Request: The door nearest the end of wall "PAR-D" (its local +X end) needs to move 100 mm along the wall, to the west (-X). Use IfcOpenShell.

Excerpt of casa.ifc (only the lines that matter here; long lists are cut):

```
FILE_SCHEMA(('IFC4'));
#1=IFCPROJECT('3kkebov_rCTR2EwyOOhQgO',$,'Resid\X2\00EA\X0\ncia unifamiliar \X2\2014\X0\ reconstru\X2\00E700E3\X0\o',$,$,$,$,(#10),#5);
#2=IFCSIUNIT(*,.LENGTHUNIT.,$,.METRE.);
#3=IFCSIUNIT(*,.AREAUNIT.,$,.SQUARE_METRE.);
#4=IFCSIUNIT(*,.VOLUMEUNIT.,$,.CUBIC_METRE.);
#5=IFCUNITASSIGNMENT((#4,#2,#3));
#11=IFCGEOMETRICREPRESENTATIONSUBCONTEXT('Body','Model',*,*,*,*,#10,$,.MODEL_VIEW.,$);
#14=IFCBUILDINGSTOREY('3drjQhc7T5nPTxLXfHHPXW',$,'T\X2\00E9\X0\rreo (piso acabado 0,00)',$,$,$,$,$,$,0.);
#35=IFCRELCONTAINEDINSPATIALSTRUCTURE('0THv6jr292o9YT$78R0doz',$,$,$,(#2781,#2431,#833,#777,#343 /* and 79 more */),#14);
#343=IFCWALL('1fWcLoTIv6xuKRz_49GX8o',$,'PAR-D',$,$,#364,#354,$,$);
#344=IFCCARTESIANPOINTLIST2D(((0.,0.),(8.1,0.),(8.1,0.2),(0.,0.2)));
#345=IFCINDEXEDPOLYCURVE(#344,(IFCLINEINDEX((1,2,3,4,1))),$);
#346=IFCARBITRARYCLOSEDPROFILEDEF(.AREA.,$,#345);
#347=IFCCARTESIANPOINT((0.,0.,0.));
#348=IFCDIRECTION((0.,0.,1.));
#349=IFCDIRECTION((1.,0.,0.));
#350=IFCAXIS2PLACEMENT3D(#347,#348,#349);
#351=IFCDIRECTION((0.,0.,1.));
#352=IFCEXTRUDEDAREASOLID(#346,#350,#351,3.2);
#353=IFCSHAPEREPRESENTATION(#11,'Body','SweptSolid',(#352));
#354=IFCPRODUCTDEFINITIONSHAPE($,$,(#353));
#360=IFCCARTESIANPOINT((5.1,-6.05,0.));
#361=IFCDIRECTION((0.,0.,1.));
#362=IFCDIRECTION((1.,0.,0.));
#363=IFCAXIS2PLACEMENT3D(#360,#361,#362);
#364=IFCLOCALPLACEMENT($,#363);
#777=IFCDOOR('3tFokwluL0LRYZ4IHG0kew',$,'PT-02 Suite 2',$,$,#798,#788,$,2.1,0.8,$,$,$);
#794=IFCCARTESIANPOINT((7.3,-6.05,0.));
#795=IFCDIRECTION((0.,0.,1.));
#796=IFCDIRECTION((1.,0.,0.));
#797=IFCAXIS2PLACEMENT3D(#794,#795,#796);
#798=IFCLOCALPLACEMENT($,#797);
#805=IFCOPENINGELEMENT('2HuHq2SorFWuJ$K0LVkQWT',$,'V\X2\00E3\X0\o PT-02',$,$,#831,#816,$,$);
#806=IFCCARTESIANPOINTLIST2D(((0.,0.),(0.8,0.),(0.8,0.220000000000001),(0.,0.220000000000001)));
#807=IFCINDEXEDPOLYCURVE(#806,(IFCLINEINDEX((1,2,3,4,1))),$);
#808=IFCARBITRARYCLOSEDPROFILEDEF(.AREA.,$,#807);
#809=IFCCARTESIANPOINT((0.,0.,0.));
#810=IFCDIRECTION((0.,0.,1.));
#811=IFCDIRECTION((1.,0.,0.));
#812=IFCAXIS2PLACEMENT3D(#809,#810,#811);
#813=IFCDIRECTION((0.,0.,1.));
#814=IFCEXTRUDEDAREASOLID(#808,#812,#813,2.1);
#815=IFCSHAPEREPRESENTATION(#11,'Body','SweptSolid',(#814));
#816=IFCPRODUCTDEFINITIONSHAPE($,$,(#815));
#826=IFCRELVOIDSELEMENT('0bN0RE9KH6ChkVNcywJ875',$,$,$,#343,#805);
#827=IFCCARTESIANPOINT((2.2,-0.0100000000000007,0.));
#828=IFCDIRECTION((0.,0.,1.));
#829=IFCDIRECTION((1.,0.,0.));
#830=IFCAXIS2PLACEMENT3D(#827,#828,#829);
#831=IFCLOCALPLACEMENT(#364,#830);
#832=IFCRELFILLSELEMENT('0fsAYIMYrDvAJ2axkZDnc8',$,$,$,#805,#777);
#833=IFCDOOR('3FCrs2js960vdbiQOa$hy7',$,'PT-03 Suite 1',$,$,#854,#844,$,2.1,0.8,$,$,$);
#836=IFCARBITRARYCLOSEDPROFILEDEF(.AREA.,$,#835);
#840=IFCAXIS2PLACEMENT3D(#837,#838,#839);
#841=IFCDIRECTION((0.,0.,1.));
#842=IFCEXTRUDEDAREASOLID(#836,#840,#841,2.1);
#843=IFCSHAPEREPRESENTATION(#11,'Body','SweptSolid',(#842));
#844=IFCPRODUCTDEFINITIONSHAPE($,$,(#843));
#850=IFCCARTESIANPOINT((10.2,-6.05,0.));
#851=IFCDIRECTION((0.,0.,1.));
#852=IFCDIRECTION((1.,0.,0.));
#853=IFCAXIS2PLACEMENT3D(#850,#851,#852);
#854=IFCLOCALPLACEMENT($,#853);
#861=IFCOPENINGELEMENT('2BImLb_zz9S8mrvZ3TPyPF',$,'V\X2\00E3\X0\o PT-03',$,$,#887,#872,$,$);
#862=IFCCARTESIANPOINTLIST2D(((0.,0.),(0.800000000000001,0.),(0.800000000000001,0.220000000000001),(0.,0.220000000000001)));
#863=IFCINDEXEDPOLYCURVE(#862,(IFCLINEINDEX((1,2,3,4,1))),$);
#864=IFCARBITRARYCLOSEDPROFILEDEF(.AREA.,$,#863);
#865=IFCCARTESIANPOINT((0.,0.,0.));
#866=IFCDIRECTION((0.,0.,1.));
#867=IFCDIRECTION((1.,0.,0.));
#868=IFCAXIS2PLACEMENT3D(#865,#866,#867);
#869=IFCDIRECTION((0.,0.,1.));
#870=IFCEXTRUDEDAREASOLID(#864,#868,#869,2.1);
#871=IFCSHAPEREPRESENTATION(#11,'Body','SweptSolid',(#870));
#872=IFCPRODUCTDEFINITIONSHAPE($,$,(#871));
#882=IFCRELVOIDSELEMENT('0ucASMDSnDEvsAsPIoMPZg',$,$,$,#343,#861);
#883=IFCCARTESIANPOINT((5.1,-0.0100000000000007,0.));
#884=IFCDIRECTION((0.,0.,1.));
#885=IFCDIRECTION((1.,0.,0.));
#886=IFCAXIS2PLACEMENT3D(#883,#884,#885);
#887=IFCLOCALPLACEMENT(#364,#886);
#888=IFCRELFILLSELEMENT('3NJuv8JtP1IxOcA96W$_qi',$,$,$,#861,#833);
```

```python
import ifcopenshell
import ifcopenshell.api.geometry
import ifcopenshell.util.placement
import ifcopenshell.util.unit

model = ifcopenshell.open("casa.ifc")
unit_scale = ifcopenshell.util.unit.calculate_unit_scale(model)

door = model.by_guid("3FCrs2js960vdbiQOa$hy7")
opening = door.FillsVoids[0].RelatingOpeningElement
wall = opening.VoidsElements[0].RelatingBuildingElement

wall_matrix = ifcopenshell.util.placement.get_local_placement(wall.ObjectPlacement)
shift = wall_matrix[:3, 0] * -0.1 / unit_scale
before = ifcopenshell.util.placement.get_local_placement(door.ObjectPlacement)[:3, 3].copy()

# The door is not placed relative to its opening, so move both.
for product in (opening, door):
    matrix = ifcopenshell.util.placement.get_local_placement(product.ObjectPlacement)
    matrix[:3, 3] += shift
    ifcopenshell.api.geometry.edit_object_placement(model, product=product, matrix=matrix, is_si=False)

after = ifcopenshell.util.placement.get_local_placement(door.ObjectPlacement)[:3, 3]
print("door moved by", (after - before).round(3) + 0.0)

model.write("casa_rev.ifc")
```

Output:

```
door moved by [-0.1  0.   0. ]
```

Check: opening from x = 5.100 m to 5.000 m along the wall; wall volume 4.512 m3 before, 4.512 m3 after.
